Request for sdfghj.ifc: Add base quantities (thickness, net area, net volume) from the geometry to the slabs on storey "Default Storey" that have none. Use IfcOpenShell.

First a look at what the model holds.

```python
import ifcopenshell
import ifcopenshell.util.element
import ifcopenshell.util.unit

model = ifcopenshell.open("sdfghj.ifc")
print(model.schema)
for unit_type in ("LENGTHUNIT", "AREAUNIT", "VOLUMEUNIT"):
    print(unit_type, ifcopenshell.util.unit.calculate_unit_scale(model, unit_type))
storey = next(s for s in model.by_type("IfcBuildingStorey") if s.Name == "Default Storey")
slabs = [e for e in ifcopenshell.util.element.get_decomposition(storey) if e.is_a("IfcSlab")]
for e in sorted(slabs, key=lambda e: e.id()):
    print(e.id(), e.is_a(), e.Name, list(ifcopenshell.util.element.get_psets(e, qtos_only=True)), sep=" | ")
```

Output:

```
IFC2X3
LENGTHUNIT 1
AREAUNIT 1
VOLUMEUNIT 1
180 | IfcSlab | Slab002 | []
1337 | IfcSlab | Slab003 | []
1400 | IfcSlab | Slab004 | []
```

```python
import ifcopenshell
import ifcopenshell.api.pset
import ifcopenshell.geom
import ifcopenshell.util.element
import ifcopenshell.util.shape
import ifcopenshell.util.unit

model = ifcopenshell.open("sdfghj.ifc")
unit_scale = ifcopenshell.util.unit.calculate_unit_scale(model)
area_scale = ifcopenshell.util.unit.calculate_unit_scale(model, "AREAUNIT")
volume_scale = ifcopenshell.util.unit.calculate_unit_scale(model, "VOLUMEUNIT")
settings = ifcopenshell.geom.settings()

storey = next(s for s in model.by_type("IfcBuildingStorey") if s.Name == "Default Storey")
slabs = [e for e in ifcopenshell.util.element.get_decomposition(storey) if e.is_a("IfcSlab")]

for e in sorted(slabs, key=lambda e: e.id()):
    if ifcopenshell.util.element.get_psets(e, qtos_only=True, should_inherit=False):
        continue
    # Geometry comes back in metres, in the element's own axes.
    shape = ifcopenshell.geom.create_shape(settings, e)
    values = {
        "Width": ifcopenshell.util.shape.get_z(shape.geometry) / unit_scale,
        "NetArea": ifcopenshell.util.shape.get_footprint_area(shape.geometry) / area_scale,
        "NetVolume": ifcopenshell.util.shape.get_volume(shape.geometry) / volume_scale,
    }
    qto = ifcopenshell.api.pset.add_qto(model, product=e, name="BaseQuantities")
    ifcopenshell.api.pset.edit_qto(model, qto=qto, properties=values)
    print(e.id(), {k: round(v, 3) for k, v in values.items()})

model.write("sdfghj_v2.ifc")
```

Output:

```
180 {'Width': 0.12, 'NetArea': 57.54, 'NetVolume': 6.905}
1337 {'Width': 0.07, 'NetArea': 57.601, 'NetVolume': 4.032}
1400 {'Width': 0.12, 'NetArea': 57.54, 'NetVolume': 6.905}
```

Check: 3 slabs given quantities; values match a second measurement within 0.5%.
